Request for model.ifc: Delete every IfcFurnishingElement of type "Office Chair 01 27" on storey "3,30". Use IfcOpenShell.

First a look at what the model holds.

```python
import ifcopenshell
import ifcopenshell.util.element

model = ifcopenshell.open("model.ifc")
print(model.schema)
storey = next(s for s in model.by_type("IfcBuildingStorey") if s.Name == "3,30")
furniture = [e for e in ifcopenshell.util.element.get_decomposition(storey) if e.is_a("IfcFurnishingElement")]
seen = {}
for e in furniture:
    element_type = ifcopenshell.util.element.get_type(e)
    name = element_type.Name if element_type not in (None, e) else None
    seen[name] = seen.get(name, 0) + 1
for name, count in sorted(seen.items(), key=str):
    print(count, "x", name)
```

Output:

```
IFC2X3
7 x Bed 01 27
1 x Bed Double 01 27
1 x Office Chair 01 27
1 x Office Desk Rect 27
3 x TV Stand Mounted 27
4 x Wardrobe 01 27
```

```python
import ifcopenshell
import ifcopenshell.api.root
import ifcopenshell.util.element

model = ifcopenshell.open("model.ifc")

storey = next(s for s in model.by_type("IfcBuildingStorey") if s.Name == "3,30")
furniture = [e for e in ifcopenshell.util.element.get_decomposition(storey) if e.is_a("IfcFurnishingElement")]
targets = [e for e in furniture if (t := ifcopenshell.util.element.get_type(e)) not in (None, e) and t.Name == "Office Chair 01 27"]

for e in targets:
    ifcopenshell.api.root.remove_product(model, product=e)
print(len(targets), "removed")

model.write("model_v2.ifc")
```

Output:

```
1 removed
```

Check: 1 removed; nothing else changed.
